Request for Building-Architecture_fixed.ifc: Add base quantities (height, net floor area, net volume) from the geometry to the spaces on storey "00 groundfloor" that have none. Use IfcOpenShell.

First a look at what the model holds.

```python
import ifcopenshell
import ifcopenshell.util.element
import ifcopenshell.util.unit

model = ifcopenshell.open("Building-Architecture_fixed.ifc")
print(model.schema)
for unit_type in ("LENGTHUNIT", "AREAUNIT", "VOLUMEUNIT"):
    print(unit_type, ifcopenshell.util.unit.calculate_unit_scale(model, unit_type))
storey = next(s for s in model.by_type("IfcBuildingStorey") if s.Name == "00 groundfloor")
spaces = [e for e in ifcopenshell.util.element.get_decomposition(storey) if e.is_a("IfcSpace")]
for e in sorted(spaces, key=lambda e: e.id()):
    print(e.id(), e.is_a(), e.Name, list(ifcopenshell.util.element.get_psets(e, qtos_only=True)), sep=" | ")
```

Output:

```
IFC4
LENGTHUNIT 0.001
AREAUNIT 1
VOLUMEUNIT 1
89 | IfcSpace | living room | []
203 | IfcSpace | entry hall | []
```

```python
import ifcopenshell
import ifcopenshell.api.pset
import ifcopenshell.geom
import ifcopenshell.util.element
import ifcopenshell.util.shape
import ifcopenshell.util.unit

model = ifcopenshell.open("Building-Architecture_fixed.ifc")
unit_scale = ifcopenshell.util.unit.calculate_unit_scale(model)
area_scale = ifcopenshell.util.unit.calculate_unit_scale(model, "AREAUNIT")
volume_scale = ifcopenshell.util.unit.calculate_unit_scale(model, "VOLUMEUNIT")
settings = ifcopenshell.geom.settings()

storey = next(s for s in model.by_type("IfcBuildingStorey") if s.Name == "00 groundfloor")
spaces = [e for e in ifcopenshell.util.element.get_decomposition(storey) if e.is_a("IfcSpace")]

for e in sorted(spaces, key=lambda e: e.id()):
    if ifcopenshell.util.element.get_psets(e, qtos_only=True, should_inherit=False):
        continue
    # Geometry comes back in metres, in the element's own axes.
    shape = ifcopenshell.geom.create_shape(settings, e)
    values = {
        "Height": ifcopenshell.util.shape.get_z(shape.geometry) / unit_scale,
        "NetFloorArea": ifcopenshell.util.shape.get_footprint_area(shape.geometry) / area_scale,
        "NetVolume": ifcopenshell.util.shape.get_volume(shape.geometry) / volume_scale,
    }
    qto = ifcopenshell.api.pset.add_qto(model, product=e, name="Qto_SpaceBaseQuantities")
    ifcopenshell.api.pset.edit_qto(model, qto=qto, properties=values)
    print(e.id(), {k: round(v, 3) for k, v in values.items()})

model.write("Building-Architecture_fixed_rev.ifc")
```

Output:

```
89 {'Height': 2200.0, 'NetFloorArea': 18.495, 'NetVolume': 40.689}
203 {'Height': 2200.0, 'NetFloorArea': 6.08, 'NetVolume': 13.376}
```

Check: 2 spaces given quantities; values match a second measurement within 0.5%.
